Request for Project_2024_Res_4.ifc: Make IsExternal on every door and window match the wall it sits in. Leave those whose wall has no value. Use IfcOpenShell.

First a look at what the model holds.

```python
import ifcopenshell
import ifcopenshell.util.element

model = ifcopenshell.open("Project_2024_Res_4.ifc")
print(model.schema)
seen = {}
for e in model.by_type("IfcDoor") + model.by_type("IfcWindow"):
    if not e.FillsVoids:
        continue
    host = e.FillsVoids[0].RelatingOpeningElement.VoidsElements[0].RelatingBuildingElement
    own = ifcopenshell.util.element.get_pset(e, f"Pset_{e.is_a()[3:].removesuffix('StandardCase')}Common", "IsExternal")
    wall = ifcopenshell.util.element.get_pset(host, "Pset_WallCommon", "IsExternal")
    seen[e.is_a(), own, wall] = seen.get((e.is_a(), own, wall), 0) + 1
for (cls, own, wall), count in sorted(seen.items(), key=str):
    print(count, cls, "IsExternal:", own, "| host wall:", wall)
```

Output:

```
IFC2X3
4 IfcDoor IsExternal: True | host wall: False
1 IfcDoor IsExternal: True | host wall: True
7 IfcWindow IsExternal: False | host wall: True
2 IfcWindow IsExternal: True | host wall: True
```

```python
import ifcopenshell
import ifcopenshell.api.pset
import ifcopenshell.util.element

model = ifcopenshell.open("Project_2024_Res_4.ifc")

count = 0
for ifc_class, pset_name in (("IfcDoor", "Pset_DoorCommon"), ("IfcWindow", "Pset_WindowCommon")):
    for e in model.by_type(ifc_class):
        if not e.FillsVoids:
            continue
        host = e.FillsVoids[0].RelatingOpeningElement.VoidsElements[0].RelatingBuildingElement
        external = ifcopenshell.util.element.get_pset(host, "Pset_WallCommon", "IsExternal")
        if external is None or ifcopenshell.util.element.get_pset(e, pset_name, "IsExternal") == external:
            continue
        pset = ifcopenshell.api.pset.add_pset(model, product=e, name=pset_name)
        ifcopenshell.api.pset.edit_pset(model, pset=pset, properties={"IsExternal": external})
        count += 1

print(count, "updated")

model.write("Project_2024_Res_4_edited.ifc")
```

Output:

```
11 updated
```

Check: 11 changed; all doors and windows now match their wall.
